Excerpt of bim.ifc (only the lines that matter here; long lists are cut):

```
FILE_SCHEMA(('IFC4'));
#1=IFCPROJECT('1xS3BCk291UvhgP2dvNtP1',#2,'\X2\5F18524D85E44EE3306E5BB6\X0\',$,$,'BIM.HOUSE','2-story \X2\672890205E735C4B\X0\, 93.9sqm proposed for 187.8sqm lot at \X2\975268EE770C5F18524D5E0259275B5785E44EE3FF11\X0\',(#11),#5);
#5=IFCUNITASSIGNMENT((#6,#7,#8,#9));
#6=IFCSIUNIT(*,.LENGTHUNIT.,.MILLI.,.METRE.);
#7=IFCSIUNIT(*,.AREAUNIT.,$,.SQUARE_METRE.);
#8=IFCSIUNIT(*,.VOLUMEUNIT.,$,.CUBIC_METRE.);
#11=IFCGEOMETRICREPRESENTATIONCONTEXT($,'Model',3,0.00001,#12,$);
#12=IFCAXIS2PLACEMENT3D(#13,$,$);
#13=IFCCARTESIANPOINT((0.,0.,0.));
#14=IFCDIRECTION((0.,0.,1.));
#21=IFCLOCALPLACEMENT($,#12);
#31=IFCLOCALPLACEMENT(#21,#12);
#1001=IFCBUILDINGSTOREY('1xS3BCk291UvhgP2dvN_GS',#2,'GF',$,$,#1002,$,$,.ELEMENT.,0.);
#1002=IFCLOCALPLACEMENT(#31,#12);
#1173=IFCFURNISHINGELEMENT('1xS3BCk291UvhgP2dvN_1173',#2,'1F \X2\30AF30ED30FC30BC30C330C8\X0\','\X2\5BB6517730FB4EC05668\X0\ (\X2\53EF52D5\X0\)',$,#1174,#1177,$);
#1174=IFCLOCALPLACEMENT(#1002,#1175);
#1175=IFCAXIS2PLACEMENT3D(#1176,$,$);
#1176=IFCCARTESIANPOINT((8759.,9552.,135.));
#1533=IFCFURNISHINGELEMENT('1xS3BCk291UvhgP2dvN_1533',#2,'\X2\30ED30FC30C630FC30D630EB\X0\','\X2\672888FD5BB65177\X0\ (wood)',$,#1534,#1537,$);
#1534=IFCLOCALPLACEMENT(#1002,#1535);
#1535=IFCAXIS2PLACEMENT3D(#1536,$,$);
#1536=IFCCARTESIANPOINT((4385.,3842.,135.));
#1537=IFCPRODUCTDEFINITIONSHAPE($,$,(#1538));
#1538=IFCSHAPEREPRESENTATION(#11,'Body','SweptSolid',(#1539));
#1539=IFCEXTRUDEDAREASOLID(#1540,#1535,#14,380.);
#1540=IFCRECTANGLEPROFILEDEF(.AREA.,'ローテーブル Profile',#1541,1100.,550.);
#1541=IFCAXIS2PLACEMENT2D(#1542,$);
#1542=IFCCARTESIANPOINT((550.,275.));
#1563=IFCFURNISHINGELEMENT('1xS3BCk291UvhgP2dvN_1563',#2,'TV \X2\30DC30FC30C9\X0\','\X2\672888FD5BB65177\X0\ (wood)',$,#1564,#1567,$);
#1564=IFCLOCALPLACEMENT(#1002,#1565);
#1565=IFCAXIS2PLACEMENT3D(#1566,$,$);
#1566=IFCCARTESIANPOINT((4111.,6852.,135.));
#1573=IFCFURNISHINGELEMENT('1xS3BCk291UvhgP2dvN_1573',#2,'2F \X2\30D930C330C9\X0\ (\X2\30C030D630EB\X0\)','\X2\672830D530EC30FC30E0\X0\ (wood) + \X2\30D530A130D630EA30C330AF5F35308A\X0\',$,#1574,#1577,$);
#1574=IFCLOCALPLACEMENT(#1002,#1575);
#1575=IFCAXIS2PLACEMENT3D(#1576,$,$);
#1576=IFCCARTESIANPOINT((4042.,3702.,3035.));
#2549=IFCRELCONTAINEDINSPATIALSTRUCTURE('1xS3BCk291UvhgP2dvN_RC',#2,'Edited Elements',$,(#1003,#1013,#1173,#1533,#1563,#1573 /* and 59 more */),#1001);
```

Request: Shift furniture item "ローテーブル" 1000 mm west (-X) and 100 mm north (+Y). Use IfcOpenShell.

```python
import ifcopenshell
import ifcopenshell.api.geometry
import ifcopenshell.util.placement
import ifcopenshell.util.unit

model = ifcopenshell.open("bim.ifc")
unit_scale = ifcopenshell.util.unit.calculate_unit_scale(model)

item = model.by_id(1533)
matrix = ifcopenshell.util.placement.get_local_placement(item.ObjectPlacement)
matrix[0, 3] -= 1 / unit_scale
matrix[1, 3] += 0.1 / unit_scale
ifcopenshell.api.geometry.edit_object_placement(model, product=item, matrix=matrix, is_si=False)

print(ifcopenshell.util.placement.get_local_placement(item.ObjectPlacement).round(3) + 0.0)

model.write("bim_v2.ifc")
```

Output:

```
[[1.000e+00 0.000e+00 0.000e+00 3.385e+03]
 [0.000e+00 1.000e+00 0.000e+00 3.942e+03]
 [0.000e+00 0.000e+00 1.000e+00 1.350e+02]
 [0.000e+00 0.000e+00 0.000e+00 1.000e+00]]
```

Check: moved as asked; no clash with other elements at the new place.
